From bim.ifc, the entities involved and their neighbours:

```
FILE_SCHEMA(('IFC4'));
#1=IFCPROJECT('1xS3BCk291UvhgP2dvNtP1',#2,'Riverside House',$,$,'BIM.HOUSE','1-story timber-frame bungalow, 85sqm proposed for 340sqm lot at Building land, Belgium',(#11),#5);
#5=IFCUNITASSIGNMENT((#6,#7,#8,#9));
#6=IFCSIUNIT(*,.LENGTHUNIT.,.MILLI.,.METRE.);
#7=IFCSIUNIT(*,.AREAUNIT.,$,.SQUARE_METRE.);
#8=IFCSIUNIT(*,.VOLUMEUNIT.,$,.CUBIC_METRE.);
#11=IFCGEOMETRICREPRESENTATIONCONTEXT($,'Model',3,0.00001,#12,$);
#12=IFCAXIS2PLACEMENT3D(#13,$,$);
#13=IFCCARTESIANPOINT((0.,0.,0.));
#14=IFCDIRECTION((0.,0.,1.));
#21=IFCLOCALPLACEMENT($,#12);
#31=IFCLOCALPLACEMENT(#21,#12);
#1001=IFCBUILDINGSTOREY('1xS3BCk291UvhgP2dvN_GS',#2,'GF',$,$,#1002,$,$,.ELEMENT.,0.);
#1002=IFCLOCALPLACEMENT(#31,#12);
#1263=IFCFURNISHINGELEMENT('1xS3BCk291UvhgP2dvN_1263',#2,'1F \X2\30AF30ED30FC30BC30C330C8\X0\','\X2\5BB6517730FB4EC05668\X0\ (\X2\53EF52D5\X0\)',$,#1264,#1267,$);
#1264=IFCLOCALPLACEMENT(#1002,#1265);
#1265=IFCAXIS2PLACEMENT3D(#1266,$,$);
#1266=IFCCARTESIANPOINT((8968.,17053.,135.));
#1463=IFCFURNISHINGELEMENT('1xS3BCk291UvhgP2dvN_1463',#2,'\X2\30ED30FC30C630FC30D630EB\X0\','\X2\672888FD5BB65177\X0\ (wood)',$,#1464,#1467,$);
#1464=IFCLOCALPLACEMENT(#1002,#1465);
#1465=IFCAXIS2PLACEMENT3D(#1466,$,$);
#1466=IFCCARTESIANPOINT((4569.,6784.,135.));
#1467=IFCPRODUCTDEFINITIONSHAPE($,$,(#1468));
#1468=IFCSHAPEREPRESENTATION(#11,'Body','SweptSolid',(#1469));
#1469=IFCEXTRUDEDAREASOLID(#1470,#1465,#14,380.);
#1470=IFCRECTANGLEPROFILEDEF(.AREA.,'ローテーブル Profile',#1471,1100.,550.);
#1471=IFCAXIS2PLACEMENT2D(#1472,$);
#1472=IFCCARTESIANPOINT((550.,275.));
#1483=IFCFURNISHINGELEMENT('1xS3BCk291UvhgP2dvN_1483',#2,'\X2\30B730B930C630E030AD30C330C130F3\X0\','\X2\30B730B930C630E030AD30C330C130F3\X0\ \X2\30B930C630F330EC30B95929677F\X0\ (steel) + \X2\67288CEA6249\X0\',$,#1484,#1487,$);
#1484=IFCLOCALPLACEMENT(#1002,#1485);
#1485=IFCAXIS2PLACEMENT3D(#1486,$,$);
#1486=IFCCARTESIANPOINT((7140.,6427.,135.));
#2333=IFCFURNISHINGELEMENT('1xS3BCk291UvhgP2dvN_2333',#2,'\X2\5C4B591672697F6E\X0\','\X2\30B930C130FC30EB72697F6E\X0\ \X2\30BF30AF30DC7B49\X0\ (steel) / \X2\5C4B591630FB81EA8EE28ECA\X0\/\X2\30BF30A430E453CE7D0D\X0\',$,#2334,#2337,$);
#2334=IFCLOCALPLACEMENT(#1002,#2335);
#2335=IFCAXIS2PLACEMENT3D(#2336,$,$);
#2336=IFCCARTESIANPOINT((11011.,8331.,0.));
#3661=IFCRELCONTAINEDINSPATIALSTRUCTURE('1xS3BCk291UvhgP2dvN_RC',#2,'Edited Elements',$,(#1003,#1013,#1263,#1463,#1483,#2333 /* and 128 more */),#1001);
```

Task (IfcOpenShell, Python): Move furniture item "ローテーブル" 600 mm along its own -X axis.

```python
import ifcopenshell
import ifcopenshell.api.geometry
import ifcopenshell.util.placement

model = ifcopenshell.open("bim.ifc")

item = model.by_guid("1xS3BCk291UvhgP2dvN_1463")
matrix = ifcopenshell.util.placement.get_local_placement(item.ObjectPlacement)
matrix[:3, 3] -= matrix[:3, 0] * 600.0
ifcopenshell.api.geometry.edit_object_placement(model, product=item, matrix=matrix, is_si=False)

print(ifcopenshell.util.placement.get_local_placement(item.ObjectPlacement).round(3) + 0.0)

model.write("bim_updated.ifc")
```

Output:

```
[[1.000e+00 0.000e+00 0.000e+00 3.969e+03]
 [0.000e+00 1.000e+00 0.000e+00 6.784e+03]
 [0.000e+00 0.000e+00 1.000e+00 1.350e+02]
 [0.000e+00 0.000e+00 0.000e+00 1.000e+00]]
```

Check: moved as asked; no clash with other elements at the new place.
